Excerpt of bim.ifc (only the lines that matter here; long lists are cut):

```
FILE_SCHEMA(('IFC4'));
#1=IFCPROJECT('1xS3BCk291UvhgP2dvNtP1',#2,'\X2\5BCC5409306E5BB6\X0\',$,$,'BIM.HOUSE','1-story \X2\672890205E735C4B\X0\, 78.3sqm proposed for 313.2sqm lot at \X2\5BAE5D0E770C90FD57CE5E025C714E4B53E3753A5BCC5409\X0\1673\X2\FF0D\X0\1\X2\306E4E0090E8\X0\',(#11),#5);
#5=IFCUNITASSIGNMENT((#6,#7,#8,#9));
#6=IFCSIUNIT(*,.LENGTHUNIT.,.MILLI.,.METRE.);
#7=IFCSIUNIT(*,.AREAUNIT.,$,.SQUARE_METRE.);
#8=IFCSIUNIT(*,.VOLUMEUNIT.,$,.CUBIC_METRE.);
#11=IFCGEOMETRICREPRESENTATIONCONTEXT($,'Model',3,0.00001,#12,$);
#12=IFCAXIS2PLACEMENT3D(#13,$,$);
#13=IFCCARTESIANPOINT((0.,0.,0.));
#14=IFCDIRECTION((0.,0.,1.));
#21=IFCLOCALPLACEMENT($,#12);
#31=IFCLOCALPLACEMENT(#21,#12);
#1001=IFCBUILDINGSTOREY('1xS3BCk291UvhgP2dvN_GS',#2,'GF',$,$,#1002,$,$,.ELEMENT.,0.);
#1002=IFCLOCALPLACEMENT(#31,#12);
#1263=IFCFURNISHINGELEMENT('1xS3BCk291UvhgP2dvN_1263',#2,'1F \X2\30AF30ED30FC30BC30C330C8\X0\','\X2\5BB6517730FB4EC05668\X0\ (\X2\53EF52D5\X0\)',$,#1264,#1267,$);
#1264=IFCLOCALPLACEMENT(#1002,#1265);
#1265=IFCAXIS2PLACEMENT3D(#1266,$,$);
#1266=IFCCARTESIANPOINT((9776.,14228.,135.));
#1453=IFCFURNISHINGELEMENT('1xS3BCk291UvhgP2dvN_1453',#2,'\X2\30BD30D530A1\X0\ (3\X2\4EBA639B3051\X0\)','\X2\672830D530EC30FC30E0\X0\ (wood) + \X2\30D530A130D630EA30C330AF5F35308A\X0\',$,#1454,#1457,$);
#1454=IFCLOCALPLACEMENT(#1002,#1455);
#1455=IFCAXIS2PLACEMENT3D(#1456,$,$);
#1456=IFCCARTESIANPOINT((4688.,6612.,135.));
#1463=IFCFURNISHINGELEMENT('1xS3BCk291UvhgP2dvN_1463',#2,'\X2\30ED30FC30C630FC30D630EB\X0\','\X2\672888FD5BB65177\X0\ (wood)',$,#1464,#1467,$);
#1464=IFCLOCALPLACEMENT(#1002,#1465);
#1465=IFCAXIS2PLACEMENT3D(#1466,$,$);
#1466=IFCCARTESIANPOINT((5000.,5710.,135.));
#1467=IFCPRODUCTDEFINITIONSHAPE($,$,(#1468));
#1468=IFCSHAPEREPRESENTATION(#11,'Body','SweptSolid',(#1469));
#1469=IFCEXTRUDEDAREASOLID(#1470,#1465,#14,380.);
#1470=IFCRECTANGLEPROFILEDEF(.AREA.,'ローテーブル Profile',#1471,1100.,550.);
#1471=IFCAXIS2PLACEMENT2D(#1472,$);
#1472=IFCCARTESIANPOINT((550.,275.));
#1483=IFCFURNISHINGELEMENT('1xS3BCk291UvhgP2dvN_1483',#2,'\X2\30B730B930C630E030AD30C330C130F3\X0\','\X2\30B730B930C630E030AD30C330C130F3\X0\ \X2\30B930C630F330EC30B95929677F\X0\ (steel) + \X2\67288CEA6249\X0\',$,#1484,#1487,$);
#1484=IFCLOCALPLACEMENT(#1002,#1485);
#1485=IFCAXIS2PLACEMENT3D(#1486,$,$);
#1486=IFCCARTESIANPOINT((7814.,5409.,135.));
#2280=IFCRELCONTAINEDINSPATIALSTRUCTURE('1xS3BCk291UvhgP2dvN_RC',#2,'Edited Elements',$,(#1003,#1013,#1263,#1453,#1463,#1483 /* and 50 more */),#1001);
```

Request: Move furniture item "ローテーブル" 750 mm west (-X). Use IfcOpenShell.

```python
import ifcopenshell
import ifcopenshell.api.geometry
import ifcopenshell.util.placement

model = ifcopenshell.open("bim.ifc")

item = model.by_guid("1xS3BCk291UvhgP2dvN_1463")
matrix = ifcopenshell.util.placement.get_local_placement(item.ObjectPlacement)
matrix[0, 3] -= 750.0
ifcopenshell.api.geometry.edit_object_placement(model, product=item, matrix=matrix, is_si=False)

print(ifcopenshell.util.placement.get_local_placement(item.ObjectPlacement).round(3) + 0.0)

model.write("bim_rev.ifc")
```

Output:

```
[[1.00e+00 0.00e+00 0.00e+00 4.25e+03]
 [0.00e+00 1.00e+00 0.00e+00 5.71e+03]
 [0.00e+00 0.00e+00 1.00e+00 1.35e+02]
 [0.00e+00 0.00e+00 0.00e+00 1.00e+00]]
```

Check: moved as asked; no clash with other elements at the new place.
